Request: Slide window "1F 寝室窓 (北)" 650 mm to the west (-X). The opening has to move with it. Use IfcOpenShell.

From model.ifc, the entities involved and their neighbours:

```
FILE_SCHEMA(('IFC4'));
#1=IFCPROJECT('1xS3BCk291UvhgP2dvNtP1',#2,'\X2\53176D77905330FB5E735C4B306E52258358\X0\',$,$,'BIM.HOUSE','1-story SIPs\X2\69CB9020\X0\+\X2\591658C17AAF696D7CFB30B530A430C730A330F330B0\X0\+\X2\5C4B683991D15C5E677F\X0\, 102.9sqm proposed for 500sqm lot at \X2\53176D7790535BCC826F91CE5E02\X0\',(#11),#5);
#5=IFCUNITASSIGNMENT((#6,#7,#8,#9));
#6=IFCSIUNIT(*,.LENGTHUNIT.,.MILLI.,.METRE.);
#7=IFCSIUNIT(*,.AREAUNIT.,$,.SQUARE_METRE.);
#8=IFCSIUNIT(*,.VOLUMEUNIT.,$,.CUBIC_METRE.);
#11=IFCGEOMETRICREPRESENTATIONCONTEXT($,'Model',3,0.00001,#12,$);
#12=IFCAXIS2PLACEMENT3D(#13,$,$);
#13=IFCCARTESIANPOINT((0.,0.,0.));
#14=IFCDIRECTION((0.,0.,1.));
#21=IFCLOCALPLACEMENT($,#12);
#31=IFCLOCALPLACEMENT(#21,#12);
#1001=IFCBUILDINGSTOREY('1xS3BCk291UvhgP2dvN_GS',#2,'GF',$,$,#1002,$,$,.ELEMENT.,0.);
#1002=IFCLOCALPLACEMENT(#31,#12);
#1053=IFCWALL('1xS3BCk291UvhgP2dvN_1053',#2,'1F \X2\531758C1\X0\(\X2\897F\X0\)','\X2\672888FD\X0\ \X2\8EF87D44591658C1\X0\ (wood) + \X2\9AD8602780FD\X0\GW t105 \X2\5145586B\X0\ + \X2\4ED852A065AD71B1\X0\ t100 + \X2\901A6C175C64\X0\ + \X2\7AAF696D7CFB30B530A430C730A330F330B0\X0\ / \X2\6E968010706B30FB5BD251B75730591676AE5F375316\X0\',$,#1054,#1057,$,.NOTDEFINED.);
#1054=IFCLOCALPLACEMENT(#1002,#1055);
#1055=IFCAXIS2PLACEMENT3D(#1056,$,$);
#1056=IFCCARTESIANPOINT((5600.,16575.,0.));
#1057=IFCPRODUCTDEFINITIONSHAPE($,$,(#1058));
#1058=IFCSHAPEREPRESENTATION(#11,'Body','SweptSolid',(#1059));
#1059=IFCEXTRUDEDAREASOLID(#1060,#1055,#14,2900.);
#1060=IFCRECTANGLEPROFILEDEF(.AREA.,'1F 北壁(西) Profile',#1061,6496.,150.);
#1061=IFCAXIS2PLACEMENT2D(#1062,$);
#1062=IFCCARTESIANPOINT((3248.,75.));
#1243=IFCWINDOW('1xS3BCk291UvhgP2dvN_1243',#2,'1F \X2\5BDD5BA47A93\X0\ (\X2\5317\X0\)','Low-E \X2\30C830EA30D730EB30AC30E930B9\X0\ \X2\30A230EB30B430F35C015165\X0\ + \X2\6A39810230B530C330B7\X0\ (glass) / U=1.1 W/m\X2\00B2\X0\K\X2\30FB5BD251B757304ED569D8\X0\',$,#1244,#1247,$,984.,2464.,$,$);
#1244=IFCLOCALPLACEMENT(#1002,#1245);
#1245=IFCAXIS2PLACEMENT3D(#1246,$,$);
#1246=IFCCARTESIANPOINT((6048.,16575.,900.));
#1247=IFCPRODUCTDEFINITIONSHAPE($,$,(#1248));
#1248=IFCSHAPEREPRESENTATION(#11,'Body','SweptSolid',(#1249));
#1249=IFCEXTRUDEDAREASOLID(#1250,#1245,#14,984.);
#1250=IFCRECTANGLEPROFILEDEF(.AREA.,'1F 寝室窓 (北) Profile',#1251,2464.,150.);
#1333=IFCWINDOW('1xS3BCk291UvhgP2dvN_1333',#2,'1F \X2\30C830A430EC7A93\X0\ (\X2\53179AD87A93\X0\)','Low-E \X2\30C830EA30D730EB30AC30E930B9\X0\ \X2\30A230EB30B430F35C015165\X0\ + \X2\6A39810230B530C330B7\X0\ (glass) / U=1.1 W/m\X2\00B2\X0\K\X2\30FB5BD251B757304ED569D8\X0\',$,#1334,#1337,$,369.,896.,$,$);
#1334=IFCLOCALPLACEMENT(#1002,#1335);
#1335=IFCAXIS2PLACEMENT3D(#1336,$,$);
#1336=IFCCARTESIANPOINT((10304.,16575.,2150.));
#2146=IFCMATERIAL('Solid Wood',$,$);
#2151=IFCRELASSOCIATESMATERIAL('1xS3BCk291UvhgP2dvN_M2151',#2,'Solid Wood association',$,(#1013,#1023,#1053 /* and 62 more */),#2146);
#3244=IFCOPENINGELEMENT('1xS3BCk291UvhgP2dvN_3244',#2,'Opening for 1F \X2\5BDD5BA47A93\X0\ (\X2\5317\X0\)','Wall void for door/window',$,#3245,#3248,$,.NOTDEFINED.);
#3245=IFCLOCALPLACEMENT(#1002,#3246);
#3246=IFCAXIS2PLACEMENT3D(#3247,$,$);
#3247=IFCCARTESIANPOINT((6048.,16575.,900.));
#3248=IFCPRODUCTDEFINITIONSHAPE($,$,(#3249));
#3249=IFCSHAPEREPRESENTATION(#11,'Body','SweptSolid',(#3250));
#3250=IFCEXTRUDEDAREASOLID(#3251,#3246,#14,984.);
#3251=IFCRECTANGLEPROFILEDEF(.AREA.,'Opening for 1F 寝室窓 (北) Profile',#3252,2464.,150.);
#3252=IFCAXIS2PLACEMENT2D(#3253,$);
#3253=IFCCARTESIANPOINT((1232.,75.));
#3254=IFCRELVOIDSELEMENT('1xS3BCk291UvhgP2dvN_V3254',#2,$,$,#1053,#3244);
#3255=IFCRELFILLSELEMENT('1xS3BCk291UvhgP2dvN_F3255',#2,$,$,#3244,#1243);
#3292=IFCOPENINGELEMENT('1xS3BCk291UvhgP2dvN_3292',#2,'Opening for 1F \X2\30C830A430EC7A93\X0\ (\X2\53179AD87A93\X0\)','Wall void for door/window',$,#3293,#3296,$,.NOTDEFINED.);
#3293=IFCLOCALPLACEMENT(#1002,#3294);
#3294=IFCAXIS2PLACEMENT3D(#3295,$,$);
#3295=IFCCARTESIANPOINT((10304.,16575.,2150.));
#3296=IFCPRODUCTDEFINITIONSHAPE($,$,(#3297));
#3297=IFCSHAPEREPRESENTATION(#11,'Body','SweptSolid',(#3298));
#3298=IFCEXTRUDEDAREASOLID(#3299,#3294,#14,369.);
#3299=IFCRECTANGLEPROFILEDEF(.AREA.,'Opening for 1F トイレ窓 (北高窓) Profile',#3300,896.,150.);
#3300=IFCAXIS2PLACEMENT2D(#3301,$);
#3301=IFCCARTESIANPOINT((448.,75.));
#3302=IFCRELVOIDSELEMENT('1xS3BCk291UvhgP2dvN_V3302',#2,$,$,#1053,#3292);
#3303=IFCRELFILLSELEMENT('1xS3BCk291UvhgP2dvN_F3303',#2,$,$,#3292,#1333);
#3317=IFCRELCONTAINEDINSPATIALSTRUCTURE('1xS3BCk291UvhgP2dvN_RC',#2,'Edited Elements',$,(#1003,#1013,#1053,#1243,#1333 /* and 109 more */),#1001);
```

```python
import ifcopenshell
import ifcopenshell.api.geometry
import ifcopenshell.util.placement

model = ifcopenshell.open("model.ifc")

window = model.by_id(1243)
opening = window.FillsVoids[0].RelatingOpeningElement
wall = opening.VoidsElements[0].RelatingBuildingElement

wall_matrix = ifcopenshell.util.placement.get_local_placement(wall.ObjectPlacement)
shift = wall_matrix[:3, 0] * -650.0
before = ifcopenshell.util.placement.get_local_placement(window.ObjectPlacement)[:3, 3].copy()

# The window is not placed relative to its opening, so move both.
for product in (opening, window):
    matrix = ifcopenshell.util.placement.get_local_placement(product.ObjectPlacement)
    matrix[:3, 3] += shift
    ifcopenshell.api.geometry.edit_object_placement(model, product=product, matrix=matrix, is_si=False)

after = ifcopenshell.util.placement.get_local_placement(window.ObjectPlacement)[:3, 3]
print("window moved by", (after - before).round(3) + 0.0)

model.write("model_edited.ifc")
```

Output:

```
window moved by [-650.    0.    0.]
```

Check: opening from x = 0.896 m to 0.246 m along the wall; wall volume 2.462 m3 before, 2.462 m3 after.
